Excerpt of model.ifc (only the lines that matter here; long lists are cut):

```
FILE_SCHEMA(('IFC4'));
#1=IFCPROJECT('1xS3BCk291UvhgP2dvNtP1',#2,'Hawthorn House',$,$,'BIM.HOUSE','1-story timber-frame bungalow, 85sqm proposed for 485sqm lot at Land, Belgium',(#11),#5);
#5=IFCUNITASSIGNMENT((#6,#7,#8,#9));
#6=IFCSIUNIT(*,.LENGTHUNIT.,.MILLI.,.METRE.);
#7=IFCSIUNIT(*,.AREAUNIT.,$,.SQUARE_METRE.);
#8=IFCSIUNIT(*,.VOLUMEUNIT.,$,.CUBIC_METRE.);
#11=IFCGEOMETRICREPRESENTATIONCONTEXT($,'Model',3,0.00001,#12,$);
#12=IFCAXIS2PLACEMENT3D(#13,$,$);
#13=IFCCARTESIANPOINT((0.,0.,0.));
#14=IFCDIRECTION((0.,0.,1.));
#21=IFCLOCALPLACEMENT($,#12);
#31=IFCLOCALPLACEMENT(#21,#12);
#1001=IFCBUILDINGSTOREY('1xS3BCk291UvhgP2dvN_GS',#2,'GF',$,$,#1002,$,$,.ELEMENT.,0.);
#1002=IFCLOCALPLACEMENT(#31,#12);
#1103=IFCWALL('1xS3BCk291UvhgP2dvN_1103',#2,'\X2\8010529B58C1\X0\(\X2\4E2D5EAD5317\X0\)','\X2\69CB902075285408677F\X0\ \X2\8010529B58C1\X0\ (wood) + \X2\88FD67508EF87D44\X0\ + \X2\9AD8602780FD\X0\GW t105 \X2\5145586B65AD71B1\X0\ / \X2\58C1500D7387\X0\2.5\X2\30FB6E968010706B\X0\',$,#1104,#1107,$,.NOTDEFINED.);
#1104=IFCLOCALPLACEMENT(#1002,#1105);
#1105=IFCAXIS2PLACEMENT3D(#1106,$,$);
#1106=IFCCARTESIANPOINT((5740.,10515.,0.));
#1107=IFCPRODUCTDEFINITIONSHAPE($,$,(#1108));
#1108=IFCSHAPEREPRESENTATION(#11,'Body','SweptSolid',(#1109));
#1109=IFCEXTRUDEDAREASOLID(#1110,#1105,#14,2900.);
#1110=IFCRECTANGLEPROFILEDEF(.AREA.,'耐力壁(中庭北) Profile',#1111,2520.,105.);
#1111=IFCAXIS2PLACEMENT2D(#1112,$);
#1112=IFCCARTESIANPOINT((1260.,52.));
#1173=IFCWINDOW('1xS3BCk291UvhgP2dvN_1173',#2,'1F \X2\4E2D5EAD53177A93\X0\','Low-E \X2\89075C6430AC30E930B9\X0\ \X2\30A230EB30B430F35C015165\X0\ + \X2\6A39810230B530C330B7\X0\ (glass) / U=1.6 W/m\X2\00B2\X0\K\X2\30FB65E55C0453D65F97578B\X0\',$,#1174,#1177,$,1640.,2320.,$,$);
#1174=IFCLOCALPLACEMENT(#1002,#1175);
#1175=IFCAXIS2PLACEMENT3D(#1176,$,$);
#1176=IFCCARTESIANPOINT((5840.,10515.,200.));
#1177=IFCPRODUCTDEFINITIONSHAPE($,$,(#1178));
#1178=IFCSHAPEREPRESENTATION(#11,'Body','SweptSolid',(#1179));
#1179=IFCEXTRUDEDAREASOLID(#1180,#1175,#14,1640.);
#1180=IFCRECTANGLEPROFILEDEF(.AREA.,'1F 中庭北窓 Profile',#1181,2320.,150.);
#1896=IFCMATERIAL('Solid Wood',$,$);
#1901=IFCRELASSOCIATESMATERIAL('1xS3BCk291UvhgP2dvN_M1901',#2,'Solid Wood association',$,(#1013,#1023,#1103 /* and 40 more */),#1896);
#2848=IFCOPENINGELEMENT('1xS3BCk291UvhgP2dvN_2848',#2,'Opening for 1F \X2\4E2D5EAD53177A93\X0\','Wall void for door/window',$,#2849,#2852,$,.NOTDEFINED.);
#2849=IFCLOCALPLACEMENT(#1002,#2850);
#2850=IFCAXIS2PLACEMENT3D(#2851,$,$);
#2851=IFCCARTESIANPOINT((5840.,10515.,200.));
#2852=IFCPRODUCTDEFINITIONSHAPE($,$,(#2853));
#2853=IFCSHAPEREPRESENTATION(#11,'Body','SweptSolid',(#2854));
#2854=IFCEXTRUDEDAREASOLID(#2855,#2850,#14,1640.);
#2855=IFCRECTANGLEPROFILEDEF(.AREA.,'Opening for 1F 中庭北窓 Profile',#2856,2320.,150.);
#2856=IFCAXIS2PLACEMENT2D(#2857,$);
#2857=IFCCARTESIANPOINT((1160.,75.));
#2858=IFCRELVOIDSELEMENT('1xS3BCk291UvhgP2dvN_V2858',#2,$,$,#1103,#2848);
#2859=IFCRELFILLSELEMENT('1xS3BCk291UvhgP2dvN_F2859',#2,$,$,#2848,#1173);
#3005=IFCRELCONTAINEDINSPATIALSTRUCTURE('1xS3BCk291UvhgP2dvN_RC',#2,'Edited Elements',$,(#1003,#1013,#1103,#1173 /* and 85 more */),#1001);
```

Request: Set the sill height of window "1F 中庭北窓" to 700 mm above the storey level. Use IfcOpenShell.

```python
import numpy as np
import ifcopenshell
import ifcopenshell.api.geometry
import ifcopenshell.geom
import ifcopenshell.util.element
import ifcopenshell.util.placement
import ifcopenshell.util.shape
import ifcopenshell.util.unit

model = ifcopenshell.open("model.ifc")
unit_scale = ifcopenshell.util.unit.calculate_unit_scale(model)

window = model.by_guid("1xS3BCk291UvhgP2dvN_1173")
opening = window.FillsVoids[0].RelatingOpeningElement
storey = ifcopenshell.util.element.get_container(window, ifc_class="IfcBuildingStorey")
level = ifcopenshell.util.placement.get_local_placement(storey.ObjectPlacement)[2, 3]

# The opening's origin need not be at the sill, so measure its lowest point.
shape = ifcopenshell.geom.create_shape(ifcopenshell.geom.settings(), opening)
bottom = ifcopenshell.util.shape.get_shape_bottom_elevation(shape, shape.geometry) / unit_scale
dz = level + 0.7 / unit_scale - bottom

shift = np.array([0.0, 0.0, dz])
# The window is not placed relative to its opening, so move both.
for product in (opening, window):
    matrix = ifcopenshell.util.placement.get_local_placement(product.ObjectPlacement)
    matrix[:3, 3] += shift
    ifcopenshell.api.geometry.edit_object_placement(model, product=product, matrix=matrix, is_si=False)

print(f"moved by {dz * unit_scale:+.3f} m")

model.write("model_edited.ifc")
```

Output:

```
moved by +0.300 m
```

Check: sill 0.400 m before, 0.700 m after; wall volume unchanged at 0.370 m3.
